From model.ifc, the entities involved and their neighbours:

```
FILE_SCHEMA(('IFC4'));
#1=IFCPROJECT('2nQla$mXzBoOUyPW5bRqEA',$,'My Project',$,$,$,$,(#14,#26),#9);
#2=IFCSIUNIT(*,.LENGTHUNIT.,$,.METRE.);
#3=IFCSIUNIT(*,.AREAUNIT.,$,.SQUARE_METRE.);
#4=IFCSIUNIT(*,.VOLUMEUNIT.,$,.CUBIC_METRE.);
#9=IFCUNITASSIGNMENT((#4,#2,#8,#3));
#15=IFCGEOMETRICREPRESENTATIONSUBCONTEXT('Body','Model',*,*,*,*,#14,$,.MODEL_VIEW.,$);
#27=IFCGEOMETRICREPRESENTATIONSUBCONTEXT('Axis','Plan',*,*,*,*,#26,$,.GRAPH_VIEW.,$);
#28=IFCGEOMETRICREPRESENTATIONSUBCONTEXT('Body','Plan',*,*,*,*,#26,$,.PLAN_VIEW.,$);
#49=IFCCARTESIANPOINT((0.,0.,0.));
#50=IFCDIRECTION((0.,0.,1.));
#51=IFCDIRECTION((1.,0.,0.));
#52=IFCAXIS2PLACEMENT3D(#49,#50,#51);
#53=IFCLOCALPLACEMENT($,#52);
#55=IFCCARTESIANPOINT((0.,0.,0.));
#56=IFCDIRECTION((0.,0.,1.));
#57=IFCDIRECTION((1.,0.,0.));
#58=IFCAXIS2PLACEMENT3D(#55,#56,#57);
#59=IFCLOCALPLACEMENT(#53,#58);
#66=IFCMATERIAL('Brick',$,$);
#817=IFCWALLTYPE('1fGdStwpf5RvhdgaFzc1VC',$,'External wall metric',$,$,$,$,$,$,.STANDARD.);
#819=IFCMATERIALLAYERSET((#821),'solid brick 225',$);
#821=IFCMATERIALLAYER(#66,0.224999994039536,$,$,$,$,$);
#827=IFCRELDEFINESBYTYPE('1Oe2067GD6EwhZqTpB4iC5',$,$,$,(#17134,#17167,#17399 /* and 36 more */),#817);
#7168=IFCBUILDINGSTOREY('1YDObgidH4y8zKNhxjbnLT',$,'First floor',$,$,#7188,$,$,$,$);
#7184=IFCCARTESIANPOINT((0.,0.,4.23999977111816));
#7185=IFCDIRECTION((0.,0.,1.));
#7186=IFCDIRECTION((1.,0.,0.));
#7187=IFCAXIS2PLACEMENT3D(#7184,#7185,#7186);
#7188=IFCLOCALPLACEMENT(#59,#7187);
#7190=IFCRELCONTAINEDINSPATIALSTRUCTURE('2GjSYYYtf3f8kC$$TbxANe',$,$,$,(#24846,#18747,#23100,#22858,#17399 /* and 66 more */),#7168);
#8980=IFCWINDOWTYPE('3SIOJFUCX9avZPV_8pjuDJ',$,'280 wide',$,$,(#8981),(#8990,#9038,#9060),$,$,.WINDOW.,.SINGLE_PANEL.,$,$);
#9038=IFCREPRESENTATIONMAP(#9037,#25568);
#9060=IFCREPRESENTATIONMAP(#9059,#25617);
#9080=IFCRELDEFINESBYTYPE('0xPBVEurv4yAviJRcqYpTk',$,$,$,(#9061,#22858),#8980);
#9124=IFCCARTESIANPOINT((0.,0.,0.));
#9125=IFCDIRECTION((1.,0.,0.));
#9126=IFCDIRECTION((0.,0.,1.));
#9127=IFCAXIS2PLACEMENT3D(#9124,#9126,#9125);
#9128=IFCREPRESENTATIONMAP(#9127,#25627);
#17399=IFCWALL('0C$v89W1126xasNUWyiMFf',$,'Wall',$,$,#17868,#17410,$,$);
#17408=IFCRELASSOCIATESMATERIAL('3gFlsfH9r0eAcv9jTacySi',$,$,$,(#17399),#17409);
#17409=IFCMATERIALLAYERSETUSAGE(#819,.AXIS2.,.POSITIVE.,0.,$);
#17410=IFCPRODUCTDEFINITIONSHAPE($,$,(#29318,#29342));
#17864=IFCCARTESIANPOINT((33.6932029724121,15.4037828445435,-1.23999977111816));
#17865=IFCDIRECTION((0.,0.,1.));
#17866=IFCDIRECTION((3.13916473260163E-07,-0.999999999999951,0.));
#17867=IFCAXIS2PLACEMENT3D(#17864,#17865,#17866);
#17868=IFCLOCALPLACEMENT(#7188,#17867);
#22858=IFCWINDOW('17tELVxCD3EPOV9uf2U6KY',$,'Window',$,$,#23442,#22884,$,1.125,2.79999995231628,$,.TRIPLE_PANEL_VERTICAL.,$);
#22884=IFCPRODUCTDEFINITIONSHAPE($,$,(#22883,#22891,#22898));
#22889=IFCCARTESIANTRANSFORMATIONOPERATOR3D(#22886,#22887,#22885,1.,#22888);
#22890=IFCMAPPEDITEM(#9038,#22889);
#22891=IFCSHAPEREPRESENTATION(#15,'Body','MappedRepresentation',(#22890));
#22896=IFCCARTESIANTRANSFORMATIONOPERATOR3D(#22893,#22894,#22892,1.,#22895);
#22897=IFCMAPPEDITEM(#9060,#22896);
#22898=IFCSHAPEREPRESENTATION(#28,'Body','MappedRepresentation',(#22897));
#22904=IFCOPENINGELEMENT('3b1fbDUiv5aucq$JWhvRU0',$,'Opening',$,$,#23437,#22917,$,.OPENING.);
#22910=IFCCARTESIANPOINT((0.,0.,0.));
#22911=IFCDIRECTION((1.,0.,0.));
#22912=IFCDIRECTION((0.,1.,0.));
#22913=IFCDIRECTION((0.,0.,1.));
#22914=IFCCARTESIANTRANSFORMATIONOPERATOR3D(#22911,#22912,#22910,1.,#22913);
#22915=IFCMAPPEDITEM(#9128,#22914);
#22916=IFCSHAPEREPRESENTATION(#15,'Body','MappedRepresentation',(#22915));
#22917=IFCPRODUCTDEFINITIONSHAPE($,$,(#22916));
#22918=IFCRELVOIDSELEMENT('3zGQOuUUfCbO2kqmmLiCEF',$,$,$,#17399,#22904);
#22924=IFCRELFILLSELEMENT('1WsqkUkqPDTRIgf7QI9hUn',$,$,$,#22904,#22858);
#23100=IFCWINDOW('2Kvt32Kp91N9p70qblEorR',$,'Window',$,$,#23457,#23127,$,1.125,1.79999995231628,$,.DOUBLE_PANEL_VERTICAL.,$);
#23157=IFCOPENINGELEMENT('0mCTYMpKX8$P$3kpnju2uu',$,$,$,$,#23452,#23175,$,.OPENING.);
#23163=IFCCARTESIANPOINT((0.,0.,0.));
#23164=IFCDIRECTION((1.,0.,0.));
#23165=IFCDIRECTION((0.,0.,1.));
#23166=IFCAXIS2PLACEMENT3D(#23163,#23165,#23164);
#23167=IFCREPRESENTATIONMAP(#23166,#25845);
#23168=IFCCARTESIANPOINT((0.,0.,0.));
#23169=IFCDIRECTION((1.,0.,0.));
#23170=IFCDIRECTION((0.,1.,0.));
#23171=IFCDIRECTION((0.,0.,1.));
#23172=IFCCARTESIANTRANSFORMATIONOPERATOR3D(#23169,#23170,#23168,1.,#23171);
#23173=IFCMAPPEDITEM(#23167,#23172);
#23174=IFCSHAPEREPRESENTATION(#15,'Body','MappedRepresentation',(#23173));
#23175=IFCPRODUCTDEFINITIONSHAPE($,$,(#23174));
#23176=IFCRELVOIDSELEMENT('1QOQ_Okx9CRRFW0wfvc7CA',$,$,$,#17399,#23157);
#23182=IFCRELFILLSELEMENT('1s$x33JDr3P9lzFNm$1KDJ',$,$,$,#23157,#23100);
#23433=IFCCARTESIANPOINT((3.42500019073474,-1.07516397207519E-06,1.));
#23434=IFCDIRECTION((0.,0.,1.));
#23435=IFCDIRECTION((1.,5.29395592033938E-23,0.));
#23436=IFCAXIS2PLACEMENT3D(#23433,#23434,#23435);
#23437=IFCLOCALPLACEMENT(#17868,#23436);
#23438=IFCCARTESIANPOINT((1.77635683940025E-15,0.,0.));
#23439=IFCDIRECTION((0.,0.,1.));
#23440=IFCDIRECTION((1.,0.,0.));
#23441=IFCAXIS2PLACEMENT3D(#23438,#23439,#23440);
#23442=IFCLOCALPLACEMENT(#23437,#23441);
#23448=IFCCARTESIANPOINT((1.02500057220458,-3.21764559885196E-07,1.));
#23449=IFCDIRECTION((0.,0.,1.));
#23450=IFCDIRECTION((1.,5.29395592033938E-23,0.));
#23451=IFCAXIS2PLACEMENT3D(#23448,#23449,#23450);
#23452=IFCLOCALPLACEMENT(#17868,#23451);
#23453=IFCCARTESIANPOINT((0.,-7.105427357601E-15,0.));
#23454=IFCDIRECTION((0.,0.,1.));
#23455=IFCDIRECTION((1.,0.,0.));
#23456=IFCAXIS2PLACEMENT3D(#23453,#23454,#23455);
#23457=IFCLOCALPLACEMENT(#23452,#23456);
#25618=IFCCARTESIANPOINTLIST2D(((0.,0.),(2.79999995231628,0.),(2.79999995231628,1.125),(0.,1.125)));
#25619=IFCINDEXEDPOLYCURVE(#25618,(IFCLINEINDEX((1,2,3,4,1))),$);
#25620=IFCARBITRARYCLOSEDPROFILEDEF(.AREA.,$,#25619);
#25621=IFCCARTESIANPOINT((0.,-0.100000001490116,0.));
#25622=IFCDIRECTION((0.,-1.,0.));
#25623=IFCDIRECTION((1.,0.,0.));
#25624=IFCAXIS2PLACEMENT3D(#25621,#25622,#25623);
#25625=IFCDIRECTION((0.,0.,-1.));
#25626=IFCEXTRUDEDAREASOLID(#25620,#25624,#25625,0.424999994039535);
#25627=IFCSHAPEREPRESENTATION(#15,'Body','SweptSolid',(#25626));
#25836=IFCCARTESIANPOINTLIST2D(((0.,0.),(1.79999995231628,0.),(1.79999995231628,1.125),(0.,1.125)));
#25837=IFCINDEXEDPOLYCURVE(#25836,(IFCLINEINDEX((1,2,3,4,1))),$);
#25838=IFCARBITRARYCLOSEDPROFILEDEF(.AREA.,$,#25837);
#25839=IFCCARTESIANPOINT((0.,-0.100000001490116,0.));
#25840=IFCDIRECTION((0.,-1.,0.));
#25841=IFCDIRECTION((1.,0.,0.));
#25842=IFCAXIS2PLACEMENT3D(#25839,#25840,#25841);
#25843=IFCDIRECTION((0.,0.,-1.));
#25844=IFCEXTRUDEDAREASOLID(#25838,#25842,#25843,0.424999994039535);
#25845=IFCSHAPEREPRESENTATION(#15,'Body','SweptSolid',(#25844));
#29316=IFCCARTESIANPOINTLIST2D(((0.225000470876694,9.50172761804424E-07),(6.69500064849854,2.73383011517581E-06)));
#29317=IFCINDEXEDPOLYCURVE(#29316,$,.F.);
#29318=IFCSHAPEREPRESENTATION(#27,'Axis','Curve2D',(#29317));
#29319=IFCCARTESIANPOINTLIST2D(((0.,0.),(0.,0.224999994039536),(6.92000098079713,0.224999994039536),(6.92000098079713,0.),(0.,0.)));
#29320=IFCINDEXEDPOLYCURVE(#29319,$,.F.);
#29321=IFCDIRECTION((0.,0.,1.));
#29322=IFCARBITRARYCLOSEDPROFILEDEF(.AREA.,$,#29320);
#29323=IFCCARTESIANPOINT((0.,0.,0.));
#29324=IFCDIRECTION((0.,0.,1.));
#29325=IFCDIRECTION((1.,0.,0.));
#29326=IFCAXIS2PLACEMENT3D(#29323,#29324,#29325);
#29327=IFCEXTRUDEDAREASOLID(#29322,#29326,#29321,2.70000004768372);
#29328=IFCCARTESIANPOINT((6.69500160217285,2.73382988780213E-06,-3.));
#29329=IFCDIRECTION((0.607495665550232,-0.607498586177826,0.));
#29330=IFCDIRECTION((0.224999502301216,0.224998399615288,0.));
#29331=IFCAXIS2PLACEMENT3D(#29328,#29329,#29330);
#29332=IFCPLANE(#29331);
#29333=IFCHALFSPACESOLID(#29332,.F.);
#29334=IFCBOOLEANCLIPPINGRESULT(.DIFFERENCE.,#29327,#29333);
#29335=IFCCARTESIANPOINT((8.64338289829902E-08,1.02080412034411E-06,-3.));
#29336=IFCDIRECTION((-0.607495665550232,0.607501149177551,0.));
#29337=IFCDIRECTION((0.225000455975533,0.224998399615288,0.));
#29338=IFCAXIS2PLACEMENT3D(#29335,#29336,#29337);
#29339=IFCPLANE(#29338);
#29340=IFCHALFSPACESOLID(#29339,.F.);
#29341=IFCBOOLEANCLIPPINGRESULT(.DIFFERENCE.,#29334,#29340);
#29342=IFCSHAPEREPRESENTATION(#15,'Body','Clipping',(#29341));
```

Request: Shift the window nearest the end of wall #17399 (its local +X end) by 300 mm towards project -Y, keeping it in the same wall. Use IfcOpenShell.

```python
import ifcopenshell
import ifcopenshell.api.geometry
import ifcopenshell.util.placement
import ifcopenshell.util.unit

model = ifcopenshell.open("model.ifc")
unit_scale = ifcopenshell.util.unit.calculate_unit_scale(model)

window = model.by_id(22858)
opening = window.FillsVoids[0].RelatingOpeningElement
wall = opening.VoidsElements[0].RelatingBuildingElement

wall_matrix = ifcopenshell.util.placement.get_local_placement(wall.ObjectPlacement)
shift = wall_matrix[:3, 0] * 0.3 / unit_scale
before = ifcopenshell.util.placement.get_local_placement(window.ObjectPlacement)[:3, 3].copy()

# The window is placed relative to its opening, so it follows when the opening moves.
matrix = ifcopenshell.util.placement.get_local_placement(opening.ObjectPlacement)
matrix[:3, 3] += shift
ifcopenshell.api.geometry.edit_object_placement(
    model, product=opening, matrix=matrix, is_si=False, should_transform_children=True
)

after = ifcopenshell.util.placement.get_local_placement(window.ObjectPlacement)[:3, 3]
print("window moved by", (after - before).round(3) + 0.0)

model.write("model-out.ifc")
```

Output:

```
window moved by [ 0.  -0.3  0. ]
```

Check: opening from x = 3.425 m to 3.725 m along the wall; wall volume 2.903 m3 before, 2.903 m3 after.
